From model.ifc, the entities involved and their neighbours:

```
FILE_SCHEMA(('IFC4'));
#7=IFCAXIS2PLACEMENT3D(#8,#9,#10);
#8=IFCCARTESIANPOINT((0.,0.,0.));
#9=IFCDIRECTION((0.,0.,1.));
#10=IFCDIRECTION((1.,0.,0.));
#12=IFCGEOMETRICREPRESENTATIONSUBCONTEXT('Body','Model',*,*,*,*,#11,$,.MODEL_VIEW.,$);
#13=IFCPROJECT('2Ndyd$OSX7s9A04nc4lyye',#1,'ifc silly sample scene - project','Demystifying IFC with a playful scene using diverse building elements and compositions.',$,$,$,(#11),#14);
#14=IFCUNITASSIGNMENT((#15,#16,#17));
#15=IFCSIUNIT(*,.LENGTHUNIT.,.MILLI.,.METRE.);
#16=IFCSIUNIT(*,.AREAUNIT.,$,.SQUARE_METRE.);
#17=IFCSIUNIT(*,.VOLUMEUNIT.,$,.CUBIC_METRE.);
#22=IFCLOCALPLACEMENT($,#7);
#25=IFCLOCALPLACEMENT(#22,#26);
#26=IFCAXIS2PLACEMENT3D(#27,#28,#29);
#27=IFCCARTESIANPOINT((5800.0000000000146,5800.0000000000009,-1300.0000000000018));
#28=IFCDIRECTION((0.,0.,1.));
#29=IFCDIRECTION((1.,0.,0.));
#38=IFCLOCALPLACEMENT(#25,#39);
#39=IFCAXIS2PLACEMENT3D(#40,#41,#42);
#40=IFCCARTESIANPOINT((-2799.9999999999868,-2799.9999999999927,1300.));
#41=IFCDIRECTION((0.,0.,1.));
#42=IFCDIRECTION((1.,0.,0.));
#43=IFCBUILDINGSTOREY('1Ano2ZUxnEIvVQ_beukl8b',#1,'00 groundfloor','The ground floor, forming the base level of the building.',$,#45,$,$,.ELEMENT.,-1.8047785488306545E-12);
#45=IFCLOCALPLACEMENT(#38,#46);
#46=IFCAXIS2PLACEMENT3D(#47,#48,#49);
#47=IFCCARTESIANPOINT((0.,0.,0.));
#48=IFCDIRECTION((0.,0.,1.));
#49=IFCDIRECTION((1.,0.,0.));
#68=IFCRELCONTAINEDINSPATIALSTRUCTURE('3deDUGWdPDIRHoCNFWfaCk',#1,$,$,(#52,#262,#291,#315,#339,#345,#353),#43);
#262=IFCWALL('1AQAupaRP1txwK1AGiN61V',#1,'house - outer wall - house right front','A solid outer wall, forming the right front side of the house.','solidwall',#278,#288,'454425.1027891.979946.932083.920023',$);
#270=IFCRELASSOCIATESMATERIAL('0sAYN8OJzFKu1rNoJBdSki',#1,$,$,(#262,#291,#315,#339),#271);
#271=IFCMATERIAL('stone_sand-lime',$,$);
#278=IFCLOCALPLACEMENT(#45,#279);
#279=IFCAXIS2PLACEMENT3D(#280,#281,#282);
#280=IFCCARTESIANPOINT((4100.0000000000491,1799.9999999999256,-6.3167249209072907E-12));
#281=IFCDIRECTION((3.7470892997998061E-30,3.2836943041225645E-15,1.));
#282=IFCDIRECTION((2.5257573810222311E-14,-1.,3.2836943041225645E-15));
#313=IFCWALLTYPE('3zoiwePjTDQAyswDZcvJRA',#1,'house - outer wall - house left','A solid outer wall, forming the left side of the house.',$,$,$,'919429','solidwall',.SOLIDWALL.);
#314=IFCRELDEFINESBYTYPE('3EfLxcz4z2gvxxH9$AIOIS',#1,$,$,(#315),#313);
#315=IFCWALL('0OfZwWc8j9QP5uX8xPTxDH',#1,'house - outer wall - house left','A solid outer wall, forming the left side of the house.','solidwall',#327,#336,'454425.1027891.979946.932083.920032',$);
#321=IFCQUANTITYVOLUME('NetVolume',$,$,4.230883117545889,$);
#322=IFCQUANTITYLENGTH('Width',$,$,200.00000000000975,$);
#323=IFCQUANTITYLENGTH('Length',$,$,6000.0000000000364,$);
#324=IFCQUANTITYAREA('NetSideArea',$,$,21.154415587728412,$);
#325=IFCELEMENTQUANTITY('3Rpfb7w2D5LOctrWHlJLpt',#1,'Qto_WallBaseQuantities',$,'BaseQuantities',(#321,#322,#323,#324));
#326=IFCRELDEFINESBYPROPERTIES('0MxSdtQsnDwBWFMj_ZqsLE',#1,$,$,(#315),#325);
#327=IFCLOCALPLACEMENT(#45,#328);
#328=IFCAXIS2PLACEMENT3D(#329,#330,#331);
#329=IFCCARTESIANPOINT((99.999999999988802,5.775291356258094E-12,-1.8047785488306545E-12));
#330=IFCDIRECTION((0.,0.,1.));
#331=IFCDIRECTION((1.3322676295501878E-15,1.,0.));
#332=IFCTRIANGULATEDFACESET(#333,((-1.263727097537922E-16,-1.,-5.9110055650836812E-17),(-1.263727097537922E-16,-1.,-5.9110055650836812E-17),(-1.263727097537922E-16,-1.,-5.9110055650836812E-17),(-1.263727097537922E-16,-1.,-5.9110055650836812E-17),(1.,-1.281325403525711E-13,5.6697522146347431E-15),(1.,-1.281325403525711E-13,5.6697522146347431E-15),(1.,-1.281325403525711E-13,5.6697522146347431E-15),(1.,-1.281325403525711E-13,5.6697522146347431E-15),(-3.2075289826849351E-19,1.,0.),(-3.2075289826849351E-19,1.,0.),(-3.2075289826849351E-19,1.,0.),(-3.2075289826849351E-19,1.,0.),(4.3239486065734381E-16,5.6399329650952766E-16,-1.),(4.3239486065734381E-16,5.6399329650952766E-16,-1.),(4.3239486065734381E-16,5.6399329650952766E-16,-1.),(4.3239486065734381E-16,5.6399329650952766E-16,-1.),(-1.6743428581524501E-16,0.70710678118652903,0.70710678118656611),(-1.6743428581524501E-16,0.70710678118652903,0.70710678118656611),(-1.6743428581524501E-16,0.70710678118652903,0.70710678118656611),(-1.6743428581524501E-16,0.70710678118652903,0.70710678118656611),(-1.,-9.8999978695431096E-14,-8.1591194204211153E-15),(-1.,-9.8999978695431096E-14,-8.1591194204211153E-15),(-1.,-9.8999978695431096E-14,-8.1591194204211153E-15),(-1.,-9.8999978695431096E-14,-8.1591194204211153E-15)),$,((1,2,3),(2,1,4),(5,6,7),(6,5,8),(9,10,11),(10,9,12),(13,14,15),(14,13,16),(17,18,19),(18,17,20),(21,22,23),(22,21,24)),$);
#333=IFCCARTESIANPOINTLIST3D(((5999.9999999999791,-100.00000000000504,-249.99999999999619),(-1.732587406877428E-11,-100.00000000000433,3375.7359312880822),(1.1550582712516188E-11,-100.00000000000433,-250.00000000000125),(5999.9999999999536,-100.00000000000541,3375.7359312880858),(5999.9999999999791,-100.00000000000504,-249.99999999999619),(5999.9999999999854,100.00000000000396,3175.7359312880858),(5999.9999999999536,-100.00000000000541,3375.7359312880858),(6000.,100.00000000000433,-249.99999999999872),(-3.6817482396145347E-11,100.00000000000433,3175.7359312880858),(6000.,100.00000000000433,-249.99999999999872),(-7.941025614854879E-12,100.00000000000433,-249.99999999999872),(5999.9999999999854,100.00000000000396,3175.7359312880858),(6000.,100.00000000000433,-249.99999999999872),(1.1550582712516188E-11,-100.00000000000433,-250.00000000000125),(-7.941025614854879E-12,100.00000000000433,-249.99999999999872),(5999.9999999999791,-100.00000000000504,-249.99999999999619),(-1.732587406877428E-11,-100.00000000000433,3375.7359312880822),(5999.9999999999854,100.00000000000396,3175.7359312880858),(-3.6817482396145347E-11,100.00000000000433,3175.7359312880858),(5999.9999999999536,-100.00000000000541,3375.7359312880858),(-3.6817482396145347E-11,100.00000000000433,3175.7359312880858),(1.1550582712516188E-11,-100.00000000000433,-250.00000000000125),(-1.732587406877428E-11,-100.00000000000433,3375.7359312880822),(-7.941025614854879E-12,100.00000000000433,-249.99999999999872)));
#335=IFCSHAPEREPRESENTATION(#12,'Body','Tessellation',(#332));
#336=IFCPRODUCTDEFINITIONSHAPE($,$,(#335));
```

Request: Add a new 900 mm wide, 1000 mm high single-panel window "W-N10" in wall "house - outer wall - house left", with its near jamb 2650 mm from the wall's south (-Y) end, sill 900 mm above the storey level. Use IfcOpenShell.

```python
import numpy as np
import ifcopenshell
import ifcopenshell.api.feature
import ifcopenshell.api.geometry
import ifcopenshell.api.pset
import ifcopenshell.api.root
import ifcopenshell.api.spatial
import ifcopenshell.geom
import ifcopenshell.util.element
import ifcopenshell.util.placement
import ifcopenshell.util.representation
import ifcopenshell.util.shape
import ifcopenshell.util.unit

model = ifcopenshell.open("model.ifc")
unit_scale = ifcopenshell.util.unit.calculate_unit_scale(model)
area_scale = ifcopenshell.util.unit.calculate_unit_scale(model, "AREAUNIT")
volume_scale = ifcopenshell.util.unit.calculate_unit_scale(model, "VOLUMEUNIT")
settings = ifcopenshell.geom.settings()


def volume(element):
    """Net volume in cubic metres, openings subtracted."""
    shape = ifcopenshell.geom.create_shape(settings, element)
    return ifcopenshell.util.shape.get_volume(shape.geometry)


wall = model.by_guid("0OfZwWc8j9QP5uX8xPTxDH")
storey = ifcopenshell.util.element.get_container(wall, ifc_class="IfcBuildingStorey")
context = ifcopenshell.util.representation.get_context(model, "Model", "Body", "MODEL_VIEW")
before = volume(wall)

width, height, from_end, sill = 0.9, 1, 2.65, 0.9  # metres

# The wall runs along its own X axis, and the end named is its -X end.
wall_shape = ifcopenshell.geom.create_shape(settings, wall)
x, y, z = ifcopenshell.util.shape.get_vertices(wall_shape.geometry).T
start = x.min() + from_end
face, thickness = float(y.min()), float(y.max() - y.min())
wall_matrix = ifcopenshell.util.placement.get_local_placement(wall.ObjectPlacement)
level = ifcopenshell.util.placement.get_local_placement(storey.ObjectPlacement)[2, 3]


def in_wall(x, y):
    """Placement at x, y metres in the wall's axes, at sill height."""
    matrix = wall_matrix.copy()
    matrix[:, 3] = wall_matrix @ np.array([x / unit_scale, y / unit_scale, 0.0, 1.0])
    matrix[2, 3] = level + sill / unit_scale
    return matrix


# Opening: a box that overshoots both wall faces by 50 mm.
opening = ifcopenshell.api.root.create_entity(model, ifc_class="IfcOpeningElement", predefined_type="OPENING")
box = ifcopenshell.api.geometry.add_wall_representation(
    model, context=context, length=width, height=height, thickness=thickness + 0.1
)
ifcopenshell.api.geometry.assign_representation(model, product=opening, representation=box)
ifcopenshell.api.geometry.edit_object_placement(model, product=opening, matrix=in_wall(start, face - 0.05), is_si=False)
ifcopenshell.api.feature.add_feature(model, feature=opening, element=wall)

window = ifcopenshell.api.root.create_entity(model, ifc_class="IfcWindow", name="W-N10", predefined_type="WINDOW")
window.OverallWidth, window.OverallHeight = width / unit_scale, height / unit_scale
window.PartitioningType = "SINGLE_PANEL"
body = ifcopenshell.api.geometry.add_window_representation(
    model,
    context=context,
    overall_width=window.OverallWidth,
    overall_height=window.OverallHeight,
    partition_type="SINGLE_PANEL",
)
ifcopenshell.api.geometry.assign_representation(model, product=window, representation=body)
ifcopenshell.api.spatial.assign_container(model, products=[window], relating_structure=storey)
ifcopenshell.api.feature.add_filling(model, opening=opening, element=window)

# Centre the window in the wall's thickness.
ifcopenshell.api.geometry.edit_object_placement(model, product=window, matrix=in_wall(start, face), is_si=False)
window_shape = ifcopenshell.geom.create_shape(settings, window)
depth = ifcopenshell.util.shape.get_vertices(window_shape.geometry)[:, 1]
offset = face + thickness / 2 - (depth.min() + depth.max()) / 2
ifcopenshell.api.geometry.edit_object_placement(model, product=window, matrix=in_wall(start, offset), is_si=False)

after = volume(wall)

# Update the wall's stored quantities.
qto = model.by_id(ifcopenshell.util.element.get_pset(wall, "Qto_WallBaseQuantities", should_inherit=False)["id"])
ifcopenshell.api.pset.edit_qto(model, qto=qto, properties={
    "NetVolume": after / volume_scale,
    "NetSideArea": after / thickness / area_scale,
})

print(f"wall volume {before:.3f} -> {after:.3f} m3")

model.write("model_v2.ifc")
```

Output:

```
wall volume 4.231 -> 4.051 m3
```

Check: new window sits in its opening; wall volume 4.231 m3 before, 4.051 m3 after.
